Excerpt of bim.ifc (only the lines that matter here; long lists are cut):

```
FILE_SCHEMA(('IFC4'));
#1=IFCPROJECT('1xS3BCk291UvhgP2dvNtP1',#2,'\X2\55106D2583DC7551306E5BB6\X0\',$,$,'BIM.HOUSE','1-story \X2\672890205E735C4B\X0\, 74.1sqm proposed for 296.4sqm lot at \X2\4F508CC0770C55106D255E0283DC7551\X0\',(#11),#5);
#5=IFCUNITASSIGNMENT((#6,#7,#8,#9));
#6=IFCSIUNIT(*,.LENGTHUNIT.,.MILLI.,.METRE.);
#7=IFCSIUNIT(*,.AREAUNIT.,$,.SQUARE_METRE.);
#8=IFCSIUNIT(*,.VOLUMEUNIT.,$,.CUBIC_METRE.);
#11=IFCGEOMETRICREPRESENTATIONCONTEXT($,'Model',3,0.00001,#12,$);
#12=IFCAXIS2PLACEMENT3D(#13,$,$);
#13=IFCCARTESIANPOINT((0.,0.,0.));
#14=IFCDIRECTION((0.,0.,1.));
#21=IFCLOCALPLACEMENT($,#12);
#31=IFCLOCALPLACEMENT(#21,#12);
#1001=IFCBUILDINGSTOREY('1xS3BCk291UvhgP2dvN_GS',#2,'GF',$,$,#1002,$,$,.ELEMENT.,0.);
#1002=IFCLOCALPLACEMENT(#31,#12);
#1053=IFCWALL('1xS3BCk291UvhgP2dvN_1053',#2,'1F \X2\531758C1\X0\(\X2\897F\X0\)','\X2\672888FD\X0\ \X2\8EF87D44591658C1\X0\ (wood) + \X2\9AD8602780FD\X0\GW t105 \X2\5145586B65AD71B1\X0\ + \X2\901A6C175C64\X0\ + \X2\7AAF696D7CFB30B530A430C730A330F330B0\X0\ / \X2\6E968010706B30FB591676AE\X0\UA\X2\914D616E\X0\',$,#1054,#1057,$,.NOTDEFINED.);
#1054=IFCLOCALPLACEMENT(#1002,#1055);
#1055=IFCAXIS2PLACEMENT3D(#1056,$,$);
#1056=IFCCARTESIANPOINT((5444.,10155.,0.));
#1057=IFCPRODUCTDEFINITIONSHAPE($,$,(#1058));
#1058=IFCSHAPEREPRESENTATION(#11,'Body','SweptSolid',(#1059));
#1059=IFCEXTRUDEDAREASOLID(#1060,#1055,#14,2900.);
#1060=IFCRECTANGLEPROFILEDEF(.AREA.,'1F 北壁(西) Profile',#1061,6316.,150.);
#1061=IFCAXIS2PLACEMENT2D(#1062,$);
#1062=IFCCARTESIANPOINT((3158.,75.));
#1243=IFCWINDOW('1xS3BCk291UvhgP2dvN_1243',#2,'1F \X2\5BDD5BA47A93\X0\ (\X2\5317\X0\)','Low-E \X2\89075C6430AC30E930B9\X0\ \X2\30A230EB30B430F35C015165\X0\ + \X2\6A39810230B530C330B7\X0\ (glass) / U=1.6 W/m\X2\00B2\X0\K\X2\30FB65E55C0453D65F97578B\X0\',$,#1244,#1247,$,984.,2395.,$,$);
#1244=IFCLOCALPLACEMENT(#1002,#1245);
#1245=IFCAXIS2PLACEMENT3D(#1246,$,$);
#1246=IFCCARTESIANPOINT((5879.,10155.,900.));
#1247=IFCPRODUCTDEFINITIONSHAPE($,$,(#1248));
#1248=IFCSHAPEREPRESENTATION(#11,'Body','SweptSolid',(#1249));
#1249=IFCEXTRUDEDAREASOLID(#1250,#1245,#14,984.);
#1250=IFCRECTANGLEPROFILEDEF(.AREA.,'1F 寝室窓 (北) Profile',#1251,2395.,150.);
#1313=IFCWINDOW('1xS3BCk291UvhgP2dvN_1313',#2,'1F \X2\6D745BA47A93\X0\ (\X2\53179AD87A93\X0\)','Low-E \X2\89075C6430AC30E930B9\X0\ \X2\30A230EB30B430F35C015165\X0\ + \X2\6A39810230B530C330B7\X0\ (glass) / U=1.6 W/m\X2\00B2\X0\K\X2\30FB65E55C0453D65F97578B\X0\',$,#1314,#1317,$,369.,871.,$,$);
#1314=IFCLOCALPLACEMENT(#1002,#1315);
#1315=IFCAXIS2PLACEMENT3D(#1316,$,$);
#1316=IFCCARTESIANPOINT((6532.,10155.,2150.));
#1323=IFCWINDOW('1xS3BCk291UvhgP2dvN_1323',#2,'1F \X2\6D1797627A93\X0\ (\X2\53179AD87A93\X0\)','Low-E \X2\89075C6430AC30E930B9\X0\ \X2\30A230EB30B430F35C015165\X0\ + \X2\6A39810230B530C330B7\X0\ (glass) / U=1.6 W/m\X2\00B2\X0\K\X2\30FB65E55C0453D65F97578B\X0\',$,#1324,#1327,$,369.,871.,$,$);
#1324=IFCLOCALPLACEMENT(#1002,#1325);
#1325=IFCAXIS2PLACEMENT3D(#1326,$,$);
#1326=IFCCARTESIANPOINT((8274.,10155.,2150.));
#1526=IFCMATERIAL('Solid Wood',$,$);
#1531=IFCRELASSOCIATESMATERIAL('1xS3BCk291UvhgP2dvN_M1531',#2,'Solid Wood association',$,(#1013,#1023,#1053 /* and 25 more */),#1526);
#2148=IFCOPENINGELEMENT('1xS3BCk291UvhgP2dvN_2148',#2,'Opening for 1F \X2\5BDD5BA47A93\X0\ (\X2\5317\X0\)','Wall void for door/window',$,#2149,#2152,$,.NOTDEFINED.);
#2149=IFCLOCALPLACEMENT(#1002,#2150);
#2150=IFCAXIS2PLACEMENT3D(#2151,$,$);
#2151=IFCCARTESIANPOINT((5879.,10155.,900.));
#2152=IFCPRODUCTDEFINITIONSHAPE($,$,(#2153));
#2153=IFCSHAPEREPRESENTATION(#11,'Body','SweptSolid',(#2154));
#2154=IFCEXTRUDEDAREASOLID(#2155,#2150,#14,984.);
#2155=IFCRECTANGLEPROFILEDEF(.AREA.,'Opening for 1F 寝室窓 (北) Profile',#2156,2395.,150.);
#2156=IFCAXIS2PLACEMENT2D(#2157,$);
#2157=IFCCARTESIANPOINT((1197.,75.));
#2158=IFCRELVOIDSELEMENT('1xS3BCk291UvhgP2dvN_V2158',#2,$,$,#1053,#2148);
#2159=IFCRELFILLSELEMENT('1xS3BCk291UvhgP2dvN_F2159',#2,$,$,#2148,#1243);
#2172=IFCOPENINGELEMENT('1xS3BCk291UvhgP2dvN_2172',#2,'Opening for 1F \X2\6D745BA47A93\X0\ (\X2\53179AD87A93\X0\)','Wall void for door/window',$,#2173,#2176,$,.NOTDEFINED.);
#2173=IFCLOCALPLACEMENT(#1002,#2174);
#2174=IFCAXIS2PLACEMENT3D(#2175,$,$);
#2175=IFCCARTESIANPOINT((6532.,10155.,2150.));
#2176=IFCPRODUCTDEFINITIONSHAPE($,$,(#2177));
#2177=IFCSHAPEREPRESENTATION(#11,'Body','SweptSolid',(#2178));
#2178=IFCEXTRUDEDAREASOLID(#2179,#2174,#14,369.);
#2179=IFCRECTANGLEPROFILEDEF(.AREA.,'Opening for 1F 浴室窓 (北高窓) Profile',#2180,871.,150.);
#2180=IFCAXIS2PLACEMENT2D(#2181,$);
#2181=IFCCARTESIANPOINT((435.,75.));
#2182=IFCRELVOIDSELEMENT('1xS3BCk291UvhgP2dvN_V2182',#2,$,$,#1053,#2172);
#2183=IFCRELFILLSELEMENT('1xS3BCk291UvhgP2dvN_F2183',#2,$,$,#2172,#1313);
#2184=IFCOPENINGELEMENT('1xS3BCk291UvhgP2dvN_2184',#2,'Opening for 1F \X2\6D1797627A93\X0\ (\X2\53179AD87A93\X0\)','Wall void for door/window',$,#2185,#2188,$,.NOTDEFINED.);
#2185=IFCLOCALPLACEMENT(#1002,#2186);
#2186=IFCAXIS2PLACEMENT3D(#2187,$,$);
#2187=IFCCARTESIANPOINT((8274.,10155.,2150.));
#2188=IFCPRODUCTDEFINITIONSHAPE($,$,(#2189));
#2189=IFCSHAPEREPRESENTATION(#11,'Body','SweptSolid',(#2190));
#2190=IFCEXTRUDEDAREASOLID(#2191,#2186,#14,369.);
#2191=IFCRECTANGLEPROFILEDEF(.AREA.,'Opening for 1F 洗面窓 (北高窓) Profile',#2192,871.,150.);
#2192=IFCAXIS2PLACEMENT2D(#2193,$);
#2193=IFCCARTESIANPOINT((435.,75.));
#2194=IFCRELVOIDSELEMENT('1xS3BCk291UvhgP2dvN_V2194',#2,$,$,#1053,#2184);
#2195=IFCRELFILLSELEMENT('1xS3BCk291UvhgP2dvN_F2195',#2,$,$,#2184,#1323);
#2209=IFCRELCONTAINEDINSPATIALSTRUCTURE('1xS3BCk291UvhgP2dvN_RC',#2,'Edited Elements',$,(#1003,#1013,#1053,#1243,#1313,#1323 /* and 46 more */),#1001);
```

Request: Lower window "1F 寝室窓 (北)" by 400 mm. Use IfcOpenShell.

```python
import numpy as np
import ifcopenshell
import ifcopenshell.api.geometry
import ifcopenshell.util.placement
import ifcopenshell.util.unit

model = ifcopenshell.open("bim.ifc")
unit_scale = ifcopenshell.util.unit.calculate_unit_scale(model)

window = model.by_guid("1xS3BCk291UvhgP2dvN_1243")
opening = window.FillsVoids[0].RelatingOpeningElement
dz = -0.4 / unit_scale

shift = np.array([0.0, 0.0, dz])
# The window is not placed relative to its opening, so move both.
for product in (opening, window):
    matrix = ifcopenshell.util.placement.get_local_placement(product.ObjectPlacement)
    matrix[:3, 3] += shift
    ifcopenshell.api.geometry.edit_object_placement(model, product=product, matrix=matrix, is_si=False)

print(f"moved by {dz * unit_scale:+.3f} m")

model.write("bim_updated.ifc")
```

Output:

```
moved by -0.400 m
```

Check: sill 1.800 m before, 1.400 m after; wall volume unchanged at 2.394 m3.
